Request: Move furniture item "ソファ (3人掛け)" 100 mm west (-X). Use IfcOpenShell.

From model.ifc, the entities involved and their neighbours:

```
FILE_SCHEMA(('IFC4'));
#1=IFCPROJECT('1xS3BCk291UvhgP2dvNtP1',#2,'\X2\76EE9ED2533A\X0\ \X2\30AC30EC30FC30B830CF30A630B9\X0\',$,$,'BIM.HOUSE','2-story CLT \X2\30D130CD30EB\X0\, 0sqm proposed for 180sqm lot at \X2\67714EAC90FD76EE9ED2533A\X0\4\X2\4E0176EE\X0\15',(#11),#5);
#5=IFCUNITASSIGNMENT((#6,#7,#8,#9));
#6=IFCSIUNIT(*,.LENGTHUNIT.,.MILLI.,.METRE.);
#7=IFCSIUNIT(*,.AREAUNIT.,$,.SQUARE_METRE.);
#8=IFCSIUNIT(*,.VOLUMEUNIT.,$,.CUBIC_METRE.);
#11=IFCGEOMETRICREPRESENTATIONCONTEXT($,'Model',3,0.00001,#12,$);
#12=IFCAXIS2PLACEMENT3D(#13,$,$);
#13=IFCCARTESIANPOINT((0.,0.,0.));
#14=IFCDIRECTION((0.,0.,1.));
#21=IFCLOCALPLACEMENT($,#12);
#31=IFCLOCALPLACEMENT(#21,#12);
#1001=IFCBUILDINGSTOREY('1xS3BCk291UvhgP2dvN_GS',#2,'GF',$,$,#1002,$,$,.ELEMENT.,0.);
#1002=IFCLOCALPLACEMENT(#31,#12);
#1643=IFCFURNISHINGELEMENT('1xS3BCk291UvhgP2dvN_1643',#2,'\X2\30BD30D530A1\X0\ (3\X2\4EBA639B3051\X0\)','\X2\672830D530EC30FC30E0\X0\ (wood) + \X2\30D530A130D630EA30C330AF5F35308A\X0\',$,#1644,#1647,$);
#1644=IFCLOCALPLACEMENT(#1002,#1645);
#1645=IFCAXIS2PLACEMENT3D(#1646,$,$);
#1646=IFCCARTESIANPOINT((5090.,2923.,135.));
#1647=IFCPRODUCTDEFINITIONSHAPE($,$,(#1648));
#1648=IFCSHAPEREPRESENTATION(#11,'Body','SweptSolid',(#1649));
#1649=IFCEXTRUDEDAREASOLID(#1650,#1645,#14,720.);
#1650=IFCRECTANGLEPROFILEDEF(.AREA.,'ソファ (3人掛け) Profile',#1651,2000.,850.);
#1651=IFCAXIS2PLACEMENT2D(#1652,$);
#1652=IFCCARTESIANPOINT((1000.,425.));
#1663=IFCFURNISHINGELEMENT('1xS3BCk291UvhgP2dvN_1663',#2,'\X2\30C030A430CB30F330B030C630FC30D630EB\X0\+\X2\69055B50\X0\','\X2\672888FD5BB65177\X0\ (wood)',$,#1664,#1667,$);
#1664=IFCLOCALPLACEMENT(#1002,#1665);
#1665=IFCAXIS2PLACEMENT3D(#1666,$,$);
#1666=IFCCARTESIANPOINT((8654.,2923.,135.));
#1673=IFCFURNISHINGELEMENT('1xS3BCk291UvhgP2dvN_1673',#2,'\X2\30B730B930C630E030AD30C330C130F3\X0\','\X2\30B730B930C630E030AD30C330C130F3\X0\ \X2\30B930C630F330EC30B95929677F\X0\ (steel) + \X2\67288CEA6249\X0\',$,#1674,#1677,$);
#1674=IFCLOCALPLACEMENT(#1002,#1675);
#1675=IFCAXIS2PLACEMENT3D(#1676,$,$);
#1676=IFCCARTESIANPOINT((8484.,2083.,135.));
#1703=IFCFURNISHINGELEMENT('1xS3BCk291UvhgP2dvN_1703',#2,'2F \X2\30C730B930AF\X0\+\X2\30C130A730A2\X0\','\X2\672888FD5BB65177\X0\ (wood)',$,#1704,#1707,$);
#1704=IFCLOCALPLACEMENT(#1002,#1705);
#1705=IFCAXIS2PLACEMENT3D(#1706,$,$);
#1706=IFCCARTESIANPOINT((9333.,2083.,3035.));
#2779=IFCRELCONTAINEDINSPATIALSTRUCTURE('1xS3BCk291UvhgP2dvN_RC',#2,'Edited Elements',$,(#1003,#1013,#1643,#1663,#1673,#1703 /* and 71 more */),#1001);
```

```python
import ifcopenshell
import ifcopenshell.api.geometry
import ifcopenshell.util.placement
import ifcopenshell.util.unit

model = ifcopenshell.open("model.ifc")
unit_scale = ifcopenshell.util.unit.calculate_unit_scale(model)

item = model.by_guid("1xS3BCk291UvhgP2dvN_1643")
matrix = ifcopenshell.util.placement.get_local_placement(item.ObjectPlacement)
matrix[0, 3] -= 0.1 / unit_scale
ifcopenshell.api.geometry.edit_object_placement(model, product=item, matrix=matrix, is_si=False)

print(ifcopenshell.util.placement.get_local_placement(item.ObjectPlacement).round(3) + 0.0)

model.write("model-out.ifc")
```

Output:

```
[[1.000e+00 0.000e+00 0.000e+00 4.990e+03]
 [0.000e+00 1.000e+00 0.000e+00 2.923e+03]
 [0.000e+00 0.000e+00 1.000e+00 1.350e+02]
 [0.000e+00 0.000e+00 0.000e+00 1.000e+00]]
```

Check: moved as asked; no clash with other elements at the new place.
